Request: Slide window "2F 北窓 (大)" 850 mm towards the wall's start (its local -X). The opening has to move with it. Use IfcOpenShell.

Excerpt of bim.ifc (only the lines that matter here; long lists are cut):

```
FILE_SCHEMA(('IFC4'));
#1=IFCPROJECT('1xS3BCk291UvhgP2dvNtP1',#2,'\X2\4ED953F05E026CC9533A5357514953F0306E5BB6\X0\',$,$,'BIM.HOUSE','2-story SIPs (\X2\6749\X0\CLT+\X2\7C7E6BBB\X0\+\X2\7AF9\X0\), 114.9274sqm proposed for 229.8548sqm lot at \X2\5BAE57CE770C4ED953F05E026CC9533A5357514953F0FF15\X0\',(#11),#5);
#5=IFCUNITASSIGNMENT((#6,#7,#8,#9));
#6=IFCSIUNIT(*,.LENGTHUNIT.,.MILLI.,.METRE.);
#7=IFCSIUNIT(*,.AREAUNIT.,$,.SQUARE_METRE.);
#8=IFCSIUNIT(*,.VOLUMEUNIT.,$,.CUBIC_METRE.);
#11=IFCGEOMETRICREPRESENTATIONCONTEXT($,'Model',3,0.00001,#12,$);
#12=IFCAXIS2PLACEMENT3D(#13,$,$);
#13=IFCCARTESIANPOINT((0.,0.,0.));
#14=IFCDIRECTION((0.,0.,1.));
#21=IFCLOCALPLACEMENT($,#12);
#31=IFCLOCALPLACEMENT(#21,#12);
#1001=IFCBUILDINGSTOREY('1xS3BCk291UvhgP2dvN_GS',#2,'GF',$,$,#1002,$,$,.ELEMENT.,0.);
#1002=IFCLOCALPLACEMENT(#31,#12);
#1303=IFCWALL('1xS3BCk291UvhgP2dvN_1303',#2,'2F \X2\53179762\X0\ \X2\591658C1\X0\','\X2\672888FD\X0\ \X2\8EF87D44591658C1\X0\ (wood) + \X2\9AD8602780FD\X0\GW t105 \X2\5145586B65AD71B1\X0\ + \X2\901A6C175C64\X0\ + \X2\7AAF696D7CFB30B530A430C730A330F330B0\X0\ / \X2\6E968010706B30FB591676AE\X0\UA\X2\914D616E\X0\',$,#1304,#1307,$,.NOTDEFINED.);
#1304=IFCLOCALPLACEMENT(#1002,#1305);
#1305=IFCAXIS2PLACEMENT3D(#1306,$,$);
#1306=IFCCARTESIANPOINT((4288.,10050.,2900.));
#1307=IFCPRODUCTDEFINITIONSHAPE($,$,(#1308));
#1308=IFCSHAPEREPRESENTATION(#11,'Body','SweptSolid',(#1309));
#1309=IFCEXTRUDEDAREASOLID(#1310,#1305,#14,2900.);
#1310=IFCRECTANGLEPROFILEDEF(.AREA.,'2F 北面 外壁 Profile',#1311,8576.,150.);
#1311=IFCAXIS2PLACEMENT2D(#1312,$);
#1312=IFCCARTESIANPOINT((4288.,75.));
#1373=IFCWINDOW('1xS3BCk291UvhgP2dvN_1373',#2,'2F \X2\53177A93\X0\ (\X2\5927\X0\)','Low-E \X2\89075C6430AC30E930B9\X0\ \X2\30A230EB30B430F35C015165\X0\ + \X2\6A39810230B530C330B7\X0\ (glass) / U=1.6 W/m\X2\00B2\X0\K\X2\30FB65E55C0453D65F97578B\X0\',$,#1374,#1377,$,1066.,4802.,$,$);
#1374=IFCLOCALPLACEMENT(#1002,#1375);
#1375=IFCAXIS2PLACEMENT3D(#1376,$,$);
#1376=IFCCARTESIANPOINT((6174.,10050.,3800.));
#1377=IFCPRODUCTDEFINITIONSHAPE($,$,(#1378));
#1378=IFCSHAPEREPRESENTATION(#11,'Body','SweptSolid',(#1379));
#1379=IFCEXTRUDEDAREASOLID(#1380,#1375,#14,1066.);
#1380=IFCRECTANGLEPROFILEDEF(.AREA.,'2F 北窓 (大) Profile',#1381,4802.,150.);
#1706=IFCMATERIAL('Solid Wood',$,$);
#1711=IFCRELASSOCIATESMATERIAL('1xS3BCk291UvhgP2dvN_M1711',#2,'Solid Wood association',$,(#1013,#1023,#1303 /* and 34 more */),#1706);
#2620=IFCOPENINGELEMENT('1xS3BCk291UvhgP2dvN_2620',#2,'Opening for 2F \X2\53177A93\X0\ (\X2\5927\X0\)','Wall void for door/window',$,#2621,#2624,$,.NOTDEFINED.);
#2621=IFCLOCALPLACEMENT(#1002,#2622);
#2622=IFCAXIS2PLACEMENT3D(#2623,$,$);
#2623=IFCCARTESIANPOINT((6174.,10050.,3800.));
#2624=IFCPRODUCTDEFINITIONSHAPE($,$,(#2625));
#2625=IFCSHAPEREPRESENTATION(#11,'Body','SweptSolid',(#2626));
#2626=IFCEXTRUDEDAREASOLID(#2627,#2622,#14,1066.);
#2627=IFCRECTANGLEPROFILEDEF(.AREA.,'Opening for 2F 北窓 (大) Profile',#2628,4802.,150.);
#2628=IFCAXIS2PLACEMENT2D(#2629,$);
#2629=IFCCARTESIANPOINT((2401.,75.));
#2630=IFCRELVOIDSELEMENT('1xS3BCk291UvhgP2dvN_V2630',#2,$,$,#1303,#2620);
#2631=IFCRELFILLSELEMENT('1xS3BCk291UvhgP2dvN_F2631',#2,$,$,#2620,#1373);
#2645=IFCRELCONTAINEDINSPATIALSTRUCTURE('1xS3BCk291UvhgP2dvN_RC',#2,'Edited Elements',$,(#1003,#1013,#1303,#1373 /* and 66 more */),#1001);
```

```python
import ifcopenshell
import ifcopenshell.api.geometry
import ifcopenshell.util.placement
import ifcopenshell.util.unit

model = ifcopenshell.open("bim.ifc")
unit_scale = ifcopenshell.util.unit.calculate_unit_scale(model)

window = model.by_guid("1xS3BCk291UvhgP2dvN_1373")
opening = window.FillsVoids[0].RelatingOpeningElement
wall = opening.VoidsElements[0].RelatingBuildingElement

wall_matrix = ifcopenshell.util.placement.get_local_placement(wall.ObjectPlacement)
shift = wall_matrix[:3, 0] * -0.85 / unit_scale
before = ifcopenshell.util.placement.get_local_placement(window.ObjectPlacement)[:3, 3].copy()

# The window is not placed relative to its opening, so move both.
for product in (opening, window):
    matrix = ifcopenshell.util.placement.get_local_placement(product.ObjectPlacement)
    matrix[:3, 3] += shift
    ifcopenshell.api.geometry.edit_object_placement(model, product=product, matrix=matrix, is_si=False)

after = ifcopenshell.util.placement.get_local_placement(window.ObjectPlacement)[:3, 3]
print("window moved by", (after - before).round(3) + 0.0)

model.write("bim_updated.ifc")
```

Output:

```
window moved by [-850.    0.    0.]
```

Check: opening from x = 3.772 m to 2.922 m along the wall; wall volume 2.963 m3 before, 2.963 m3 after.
